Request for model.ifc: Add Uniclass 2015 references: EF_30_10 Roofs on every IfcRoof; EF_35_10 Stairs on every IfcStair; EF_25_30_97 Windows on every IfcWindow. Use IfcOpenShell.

First a look at what the model holds.

```python
import ifcopenshell

model = ifcopenshell.open("model.ifc")
print(model.schema)
print("classifications:", [c.Name for c in model.by_type("IfcClassification")])
for ifc_class in ("IfcDoor", "IfcRoof", "IfcStair", "IfcWall", "IfcWindow"):
    print(ifc_class, len(model.by_type(ifc_class)))
```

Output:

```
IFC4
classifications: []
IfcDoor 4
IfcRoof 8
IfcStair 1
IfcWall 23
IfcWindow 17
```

```python
import ifcopenshell
import ifcopenshell.api.classification

model = ifcopenshell.open("model.ifc")

system = ifcopenshell.api.classification.add_classification(model, classification="Uniclass 2015")

codes = {
    "IfcRoof": ("EF_30_10", "Roofs"),
    "IfcStair": ("EF_35_10", "Stairs"),
    "IfcWindow": ("EF_25_30_97", "Windows"),
}
for ifc_class, (code, name) in codes.items():
    products = model.by_type(ifc_class)
    ifcopenshell.api.classification.add_reference(
        model, products=products, classification=system, identification=code, name=name
    )
    print(code, len(products))

model.write("model_v2.ifc")
```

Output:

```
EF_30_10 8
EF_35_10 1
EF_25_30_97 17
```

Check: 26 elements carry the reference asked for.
